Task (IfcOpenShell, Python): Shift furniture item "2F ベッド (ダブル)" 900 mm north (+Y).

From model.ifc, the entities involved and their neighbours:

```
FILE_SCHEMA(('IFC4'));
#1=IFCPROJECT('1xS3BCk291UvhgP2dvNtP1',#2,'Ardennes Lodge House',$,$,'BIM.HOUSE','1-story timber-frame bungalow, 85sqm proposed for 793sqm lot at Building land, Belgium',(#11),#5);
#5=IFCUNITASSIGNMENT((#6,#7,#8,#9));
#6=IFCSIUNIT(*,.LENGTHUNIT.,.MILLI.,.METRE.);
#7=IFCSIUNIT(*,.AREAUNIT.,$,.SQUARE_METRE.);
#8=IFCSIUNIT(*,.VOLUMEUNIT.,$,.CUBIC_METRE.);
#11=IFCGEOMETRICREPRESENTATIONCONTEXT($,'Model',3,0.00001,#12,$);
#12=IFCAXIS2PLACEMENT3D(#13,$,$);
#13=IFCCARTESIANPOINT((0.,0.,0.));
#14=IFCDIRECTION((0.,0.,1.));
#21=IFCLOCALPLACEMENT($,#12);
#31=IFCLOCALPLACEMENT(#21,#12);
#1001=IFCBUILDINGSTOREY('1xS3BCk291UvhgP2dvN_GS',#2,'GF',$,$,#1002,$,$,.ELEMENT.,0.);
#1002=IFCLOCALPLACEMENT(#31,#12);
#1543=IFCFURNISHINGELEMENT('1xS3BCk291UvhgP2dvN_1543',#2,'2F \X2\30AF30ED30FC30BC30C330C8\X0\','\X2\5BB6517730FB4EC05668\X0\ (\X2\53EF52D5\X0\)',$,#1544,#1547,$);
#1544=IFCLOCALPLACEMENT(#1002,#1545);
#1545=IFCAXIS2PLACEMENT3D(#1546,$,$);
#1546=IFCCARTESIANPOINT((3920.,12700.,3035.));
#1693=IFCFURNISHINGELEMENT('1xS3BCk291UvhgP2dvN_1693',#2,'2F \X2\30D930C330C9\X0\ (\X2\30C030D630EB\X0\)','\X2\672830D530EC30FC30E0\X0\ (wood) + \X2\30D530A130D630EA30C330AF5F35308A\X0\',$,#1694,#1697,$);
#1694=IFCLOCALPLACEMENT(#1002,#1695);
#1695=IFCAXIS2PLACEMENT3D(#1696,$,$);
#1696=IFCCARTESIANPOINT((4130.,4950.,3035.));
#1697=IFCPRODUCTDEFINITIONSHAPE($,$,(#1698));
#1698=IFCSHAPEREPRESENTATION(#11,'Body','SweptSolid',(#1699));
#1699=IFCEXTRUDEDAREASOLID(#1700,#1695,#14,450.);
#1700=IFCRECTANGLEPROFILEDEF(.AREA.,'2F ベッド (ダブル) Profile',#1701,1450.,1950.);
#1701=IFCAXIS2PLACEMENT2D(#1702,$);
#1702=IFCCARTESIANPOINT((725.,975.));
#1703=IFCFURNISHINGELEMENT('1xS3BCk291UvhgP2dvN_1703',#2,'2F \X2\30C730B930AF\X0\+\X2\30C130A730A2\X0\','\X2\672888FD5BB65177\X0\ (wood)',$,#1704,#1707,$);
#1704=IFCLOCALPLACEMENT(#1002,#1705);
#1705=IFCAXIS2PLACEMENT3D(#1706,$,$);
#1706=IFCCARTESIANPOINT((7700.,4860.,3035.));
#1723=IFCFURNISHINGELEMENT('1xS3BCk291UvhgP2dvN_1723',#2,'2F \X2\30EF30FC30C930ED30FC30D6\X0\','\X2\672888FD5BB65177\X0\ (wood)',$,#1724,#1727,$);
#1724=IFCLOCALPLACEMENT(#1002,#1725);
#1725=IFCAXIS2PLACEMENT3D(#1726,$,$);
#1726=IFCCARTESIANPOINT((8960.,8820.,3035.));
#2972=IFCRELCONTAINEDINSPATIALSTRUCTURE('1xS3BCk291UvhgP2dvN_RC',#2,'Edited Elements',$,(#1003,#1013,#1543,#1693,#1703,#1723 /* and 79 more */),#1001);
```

```python
import ifcopenshell
import ifcopenshell.api.geometry
import ifcopenshell.util.placement

model = ifcopenshell.open("model.ifc")

item = model.by_id(1693)
matrix = ifcopenshell.util.placement.get_local_placement(item.ObjectPlacement)
matrix[1, 3] += 900.0
ifcopenshell.api.geometry.edit_object_placement(model, product=item, matrix=matrix, is_si=False)

print(ifcopenshell.util.placement.get_local_placement(item.ObjectPlacement).round(3) + 0.0)

model.write("model-out.ifc")
```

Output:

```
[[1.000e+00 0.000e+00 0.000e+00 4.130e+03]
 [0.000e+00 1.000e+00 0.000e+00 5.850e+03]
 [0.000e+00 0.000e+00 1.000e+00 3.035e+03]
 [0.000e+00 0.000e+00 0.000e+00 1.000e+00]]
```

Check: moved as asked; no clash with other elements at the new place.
